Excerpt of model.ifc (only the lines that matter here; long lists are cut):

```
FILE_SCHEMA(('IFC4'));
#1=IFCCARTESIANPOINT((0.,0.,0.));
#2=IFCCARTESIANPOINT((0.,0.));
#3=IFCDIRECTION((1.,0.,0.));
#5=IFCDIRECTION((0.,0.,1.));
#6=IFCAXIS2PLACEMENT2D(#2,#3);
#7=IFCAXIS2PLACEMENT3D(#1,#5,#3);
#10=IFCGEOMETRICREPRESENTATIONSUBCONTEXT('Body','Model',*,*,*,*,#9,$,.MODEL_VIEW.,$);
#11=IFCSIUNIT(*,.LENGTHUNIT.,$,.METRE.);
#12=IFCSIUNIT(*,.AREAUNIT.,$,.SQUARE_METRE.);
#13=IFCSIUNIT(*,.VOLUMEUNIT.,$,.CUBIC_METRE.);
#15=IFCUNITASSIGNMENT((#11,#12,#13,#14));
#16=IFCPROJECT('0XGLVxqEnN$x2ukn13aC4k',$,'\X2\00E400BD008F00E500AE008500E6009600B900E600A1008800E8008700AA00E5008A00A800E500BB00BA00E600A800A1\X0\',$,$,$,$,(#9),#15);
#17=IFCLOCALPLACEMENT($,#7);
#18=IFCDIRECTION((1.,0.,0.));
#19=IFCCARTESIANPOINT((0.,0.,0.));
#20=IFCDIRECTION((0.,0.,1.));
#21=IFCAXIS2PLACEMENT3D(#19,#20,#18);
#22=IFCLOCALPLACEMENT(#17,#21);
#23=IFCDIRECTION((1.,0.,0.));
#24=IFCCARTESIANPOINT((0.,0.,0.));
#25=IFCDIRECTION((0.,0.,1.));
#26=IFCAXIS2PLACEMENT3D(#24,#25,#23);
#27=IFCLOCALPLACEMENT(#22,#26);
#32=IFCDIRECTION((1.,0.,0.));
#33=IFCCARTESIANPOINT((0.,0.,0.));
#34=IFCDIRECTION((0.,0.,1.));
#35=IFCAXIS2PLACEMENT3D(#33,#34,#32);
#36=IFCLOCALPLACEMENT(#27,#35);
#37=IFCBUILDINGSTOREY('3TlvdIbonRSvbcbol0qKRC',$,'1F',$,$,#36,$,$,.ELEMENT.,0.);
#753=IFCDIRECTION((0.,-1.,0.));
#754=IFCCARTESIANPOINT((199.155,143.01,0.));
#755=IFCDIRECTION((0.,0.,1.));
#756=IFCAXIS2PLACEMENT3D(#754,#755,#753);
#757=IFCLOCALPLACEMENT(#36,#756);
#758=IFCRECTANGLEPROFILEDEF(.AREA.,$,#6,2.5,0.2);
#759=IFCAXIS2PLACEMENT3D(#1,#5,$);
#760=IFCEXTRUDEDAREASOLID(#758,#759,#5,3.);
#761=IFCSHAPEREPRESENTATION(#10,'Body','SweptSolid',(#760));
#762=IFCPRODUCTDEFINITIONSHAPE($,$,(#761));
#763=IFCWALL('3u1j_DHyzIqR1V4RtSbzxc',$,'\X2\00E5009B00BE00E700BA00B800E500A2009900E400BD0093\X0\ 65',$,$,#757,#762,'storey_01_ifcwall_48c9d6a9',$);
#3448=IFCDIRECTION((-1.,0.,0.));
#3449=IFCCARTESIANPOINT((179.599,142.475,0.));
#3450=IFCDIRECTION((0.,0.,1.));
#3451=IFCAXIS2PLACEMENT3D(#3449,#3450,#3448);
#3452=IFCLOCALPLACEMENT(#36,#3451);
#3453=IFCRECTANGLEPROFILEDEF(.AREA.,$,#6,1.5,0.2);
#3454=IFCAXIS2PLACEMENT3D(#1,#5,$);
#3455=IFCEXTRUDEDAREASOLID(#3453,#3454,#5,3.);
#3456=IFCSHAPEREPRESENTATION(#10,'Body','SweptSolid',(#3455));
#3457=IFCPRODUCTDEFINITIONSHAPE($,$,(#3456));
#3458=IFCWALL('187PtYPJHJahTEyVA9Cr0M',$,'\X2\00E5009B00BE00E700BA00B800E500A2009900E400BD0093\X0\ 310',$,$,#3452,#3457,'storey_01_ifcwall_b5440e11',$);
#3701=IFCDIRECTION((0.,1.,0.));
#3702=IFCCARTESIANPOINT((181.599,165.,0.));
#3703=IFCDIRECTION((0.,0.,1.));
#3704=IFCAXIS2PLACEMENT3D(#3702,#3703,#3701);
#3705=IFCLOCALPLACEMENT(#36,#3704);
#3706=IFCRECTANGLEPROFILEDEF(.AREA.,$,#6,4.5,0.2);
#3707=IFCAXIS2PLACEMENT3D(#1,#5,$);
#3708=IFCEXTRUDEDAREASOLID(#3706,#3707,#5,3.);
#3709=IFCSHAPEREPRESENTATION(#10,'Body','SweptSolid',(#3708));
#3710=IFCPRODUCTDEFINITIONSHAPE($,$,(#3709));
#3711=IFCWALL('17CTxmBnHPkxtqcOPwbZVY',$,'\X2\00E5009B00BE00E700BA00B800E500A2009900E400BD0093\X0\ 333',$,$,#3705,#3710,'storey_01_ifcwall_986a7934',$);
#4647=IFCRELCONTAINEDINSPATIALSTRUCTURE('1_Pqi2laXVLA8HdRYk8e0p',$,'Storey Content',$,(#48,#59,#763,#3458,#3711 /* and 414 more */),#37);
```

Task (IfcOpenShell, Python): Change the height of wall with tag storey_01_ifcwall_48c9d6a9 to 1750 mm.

```python
import ifcopenshell
import ifcopenshell.geom
import ifcopenshell.util.representation
import ifcopenshell.util.shape
import ifcopenshell.util.unit

model = ifcopenshell.open("model.ifc")
unit_scale = ifcopenshell.util.unit.calculate_unit_scale(model)
settings = ifcopenshell.geom.settings()


def volume(element):
    """Net volume in cubic metres, openings subtracted."""
    shape = ifcopenshell.geom.create_shape(settings, element)
    return ifcopenshell.util.shape.get_volume(shape.geometry)


wall = model.by_id(763)
before = volume(wall)

body = ifcopenshell.util.representation.get_representation(wall, "Model", "Body")
solid = body.Items[0]
old_height = solid.Depth
solid.Depth = 1.75 / unit_scale
after = volume(wall)

print(f"height {old_height:g} -> {solid.Depth:g}, volume {before:.3f} -> {after:.3f} m3")

model.write("model-out.ifc")
```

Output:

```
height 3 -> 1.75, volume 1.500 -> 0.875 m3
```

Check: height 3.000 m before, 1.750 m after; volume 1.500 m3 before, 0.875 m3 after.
